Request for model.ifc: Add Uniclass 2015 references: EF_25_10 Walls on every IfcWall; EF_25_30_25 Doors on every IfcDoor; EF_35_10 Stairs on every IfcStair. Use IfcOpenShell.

First a look at what the model holds.

```python
import ifcopenshell

model = ifcopenshell.open("model.ifc")
print(model.schema)
print("classifications:", [c.Name for c in model.by_type("IfcClassification")])
for ifc_class in ("IfcDoor", "IfcRoof", "IfcStair", "IfcWall", "IfcWindow"):
    print(ifc_class, len(model.by_type(ifc_class)))
```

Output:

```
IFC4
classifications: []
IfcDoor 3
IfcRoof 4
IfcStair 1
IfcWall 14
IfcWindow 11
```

```python
import ifcopenshell
import ifcopenshell.api.classification

model = ifcopenshell.open("model.ifc")

system = ifcopenshell.api.classification.add_classification(model, classification="Uniclass 2015")

codes = {
    "IfcWall": ("EF_25_10", "Walls"),
    "IfcDoor": ("EF_25_30_25", "Doors"),
    "IfcStair": ("EF_35_10", "Stairs"),
}
for ifc_class, (code, name) in codes.items():
    products = model.by_type(ifc_class)
    ifcopenshell.api.classification.add_reference(
        model, products=products, classification=system, identification=code, name=name
    )
    print(code, len(products))

model.write("model_v2.ifc")
```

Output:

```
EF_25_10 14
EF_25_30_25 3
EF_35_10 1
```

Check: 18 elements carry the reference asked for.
